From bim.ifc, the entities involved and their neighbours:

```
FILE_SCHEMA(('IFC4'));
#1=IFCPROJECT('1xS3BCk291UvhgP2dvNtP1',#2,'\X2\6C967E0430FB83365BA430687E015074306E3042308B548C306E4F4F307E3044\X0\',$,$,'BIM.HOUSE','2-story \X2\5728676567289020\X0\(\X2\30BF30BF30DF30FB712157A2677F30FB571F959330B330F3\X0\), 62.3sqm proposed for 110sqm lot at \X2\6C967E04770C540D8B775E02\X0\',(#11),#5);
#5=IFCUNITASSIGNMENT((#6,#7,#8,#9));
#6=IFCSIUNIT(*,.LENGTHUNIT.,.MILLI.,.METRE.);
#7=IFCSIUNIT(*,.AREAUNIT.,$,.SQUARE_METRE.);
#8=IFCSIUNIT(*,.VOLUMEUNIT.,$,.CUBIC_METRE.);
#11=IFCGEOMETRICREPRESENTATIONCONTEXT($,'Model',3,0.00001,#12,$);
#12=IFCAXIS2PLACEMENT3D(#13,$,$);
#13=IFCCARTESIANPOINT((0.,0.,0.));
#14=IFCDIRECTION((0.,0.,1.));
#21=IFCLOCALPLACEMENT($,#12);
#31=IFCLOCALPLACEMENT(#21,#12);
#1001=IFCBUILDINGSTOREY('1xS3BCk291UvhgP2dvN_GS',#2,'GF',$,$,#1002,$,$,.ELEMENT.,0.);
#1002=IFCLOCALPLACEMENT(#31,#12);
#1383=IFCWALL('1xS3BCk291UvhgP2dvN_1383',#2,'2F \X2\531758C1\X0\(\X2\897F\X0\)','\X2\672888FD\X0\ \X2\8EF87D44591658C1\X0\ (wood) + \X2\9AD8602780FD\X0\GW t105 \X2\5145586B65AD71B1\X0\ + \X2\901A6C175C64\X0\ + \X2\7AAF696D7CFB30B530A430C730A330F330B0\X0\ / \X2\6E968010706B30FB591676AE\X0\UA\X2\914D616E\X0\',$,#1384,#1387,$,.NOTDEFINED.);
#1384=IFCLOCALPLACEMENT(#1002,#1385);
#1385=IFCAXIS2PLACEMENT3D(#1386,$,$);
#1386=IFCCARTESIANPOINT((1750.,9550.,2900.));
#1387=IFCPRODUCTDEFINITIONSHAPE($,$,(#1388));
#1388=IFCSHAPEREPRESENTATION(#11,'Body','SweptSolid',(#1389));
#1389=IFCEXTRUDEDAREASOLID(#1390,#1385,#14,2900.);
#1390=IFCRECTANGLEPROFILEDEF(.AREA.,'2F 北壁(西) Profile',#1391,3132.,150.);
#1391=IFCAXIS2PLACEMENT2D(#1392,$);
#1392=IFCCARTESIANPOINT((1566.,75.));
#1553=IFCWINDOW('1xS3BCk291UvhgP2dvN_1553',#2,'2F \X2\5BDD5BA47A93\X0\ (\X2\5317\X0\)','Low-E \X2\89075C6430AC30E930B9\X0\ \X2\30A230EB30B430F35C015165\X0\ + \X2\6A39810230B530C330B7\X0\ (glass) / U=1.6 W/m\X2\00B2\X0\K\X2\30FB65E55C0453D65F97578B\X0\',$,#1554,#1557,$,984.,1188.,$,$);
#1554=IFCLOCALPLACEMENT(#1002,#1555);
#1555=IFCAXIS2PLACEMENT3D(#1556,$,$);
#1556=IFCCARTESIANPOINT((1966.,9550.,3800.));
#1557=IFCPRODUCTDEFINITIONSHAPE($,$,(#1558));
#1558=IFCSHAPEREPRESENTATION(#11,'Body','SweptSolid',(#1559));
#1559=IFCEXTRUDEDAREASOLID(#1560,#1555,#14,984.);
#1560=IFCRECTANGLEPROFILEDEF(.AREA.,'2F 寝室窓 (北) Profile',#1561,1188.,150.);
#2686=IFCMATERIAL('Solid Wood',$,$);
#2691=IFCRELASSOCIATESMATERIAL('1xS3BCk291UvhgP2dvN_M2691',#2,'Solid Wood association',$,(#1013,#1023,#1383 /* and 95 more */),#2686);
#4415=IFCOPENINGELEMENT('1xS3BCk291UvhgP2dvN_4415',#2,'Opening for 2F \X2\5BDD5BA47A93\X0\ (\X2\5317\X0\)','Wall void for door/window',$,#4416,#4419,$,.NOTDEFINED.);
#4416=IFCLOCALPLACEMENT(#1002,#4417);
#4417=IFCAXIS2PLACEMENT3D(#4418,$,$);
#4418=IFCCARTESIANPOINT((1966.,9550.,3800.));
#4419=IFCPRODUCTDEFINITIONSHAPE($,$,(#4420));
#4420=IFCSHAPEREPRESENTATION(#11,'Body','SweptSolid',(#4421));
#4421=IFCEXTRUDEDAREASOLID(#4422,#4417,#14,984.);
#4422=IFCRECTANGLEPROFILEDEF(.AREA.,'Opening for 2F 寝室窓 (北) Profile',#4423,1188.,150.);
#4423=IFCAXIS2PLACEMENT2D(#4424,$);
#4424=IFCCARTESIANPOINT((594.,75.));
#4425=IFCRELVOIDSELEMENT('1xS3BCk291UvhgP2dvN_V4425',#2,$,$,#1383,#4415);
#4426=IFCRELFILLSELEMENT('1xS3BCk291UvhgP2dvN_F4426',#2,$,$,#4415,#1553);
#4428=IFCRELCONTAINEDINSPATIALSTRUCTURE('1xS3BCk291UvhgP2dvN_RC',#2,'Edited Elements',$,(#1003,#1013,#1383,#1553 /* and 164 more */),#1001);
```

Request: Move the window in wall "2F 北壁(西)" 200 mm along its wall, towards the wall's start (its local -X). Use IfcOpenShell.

```python
import ifcopenshell
import ifcopenshell.api.geometry
import ifcopenshell.util.placement

model = ifcopenshell.open("bim.ifc")

window = model.by_guid("1xS3BCk291UvhgP2dvN_1553")
opening = window.FillsVoids[0].RelatingOpeningElement
wall = opening.VoidsElements[0].RelatingBuildingElement

wall_matrix = ifcopenshell.util.placement.get_local_placement(wall.ObjectPlacement)
shift = wall_matrix[:3, 0] * -200.0
before = ifcopenshell.util.placement.get_local_placement(window.ObjectPlacement)[:3, 3].copy()

# The window is not placed relative to its opening, so move both.
for product in (opening, window):
    matrix = ifcopenshell.util.placement.get_local_placement(product.ObjectPlacement)
    matrix[:3, 3] += shift
    ifcopenshell.api.geometry.edit_object_placement(model, product=product, matrix=matrix, is_si=False)

after = ifcopenshell.util.placement.get_local_placement(window.ObjectPlacement)[:3, 3]
print("window moved by", (after - before).round(3) + 0.0)

model.write("bim_rev.ifc")
```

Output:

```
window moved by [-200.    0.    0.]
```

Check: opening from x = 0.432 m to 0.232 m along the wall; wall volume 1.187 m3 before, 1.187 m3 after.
